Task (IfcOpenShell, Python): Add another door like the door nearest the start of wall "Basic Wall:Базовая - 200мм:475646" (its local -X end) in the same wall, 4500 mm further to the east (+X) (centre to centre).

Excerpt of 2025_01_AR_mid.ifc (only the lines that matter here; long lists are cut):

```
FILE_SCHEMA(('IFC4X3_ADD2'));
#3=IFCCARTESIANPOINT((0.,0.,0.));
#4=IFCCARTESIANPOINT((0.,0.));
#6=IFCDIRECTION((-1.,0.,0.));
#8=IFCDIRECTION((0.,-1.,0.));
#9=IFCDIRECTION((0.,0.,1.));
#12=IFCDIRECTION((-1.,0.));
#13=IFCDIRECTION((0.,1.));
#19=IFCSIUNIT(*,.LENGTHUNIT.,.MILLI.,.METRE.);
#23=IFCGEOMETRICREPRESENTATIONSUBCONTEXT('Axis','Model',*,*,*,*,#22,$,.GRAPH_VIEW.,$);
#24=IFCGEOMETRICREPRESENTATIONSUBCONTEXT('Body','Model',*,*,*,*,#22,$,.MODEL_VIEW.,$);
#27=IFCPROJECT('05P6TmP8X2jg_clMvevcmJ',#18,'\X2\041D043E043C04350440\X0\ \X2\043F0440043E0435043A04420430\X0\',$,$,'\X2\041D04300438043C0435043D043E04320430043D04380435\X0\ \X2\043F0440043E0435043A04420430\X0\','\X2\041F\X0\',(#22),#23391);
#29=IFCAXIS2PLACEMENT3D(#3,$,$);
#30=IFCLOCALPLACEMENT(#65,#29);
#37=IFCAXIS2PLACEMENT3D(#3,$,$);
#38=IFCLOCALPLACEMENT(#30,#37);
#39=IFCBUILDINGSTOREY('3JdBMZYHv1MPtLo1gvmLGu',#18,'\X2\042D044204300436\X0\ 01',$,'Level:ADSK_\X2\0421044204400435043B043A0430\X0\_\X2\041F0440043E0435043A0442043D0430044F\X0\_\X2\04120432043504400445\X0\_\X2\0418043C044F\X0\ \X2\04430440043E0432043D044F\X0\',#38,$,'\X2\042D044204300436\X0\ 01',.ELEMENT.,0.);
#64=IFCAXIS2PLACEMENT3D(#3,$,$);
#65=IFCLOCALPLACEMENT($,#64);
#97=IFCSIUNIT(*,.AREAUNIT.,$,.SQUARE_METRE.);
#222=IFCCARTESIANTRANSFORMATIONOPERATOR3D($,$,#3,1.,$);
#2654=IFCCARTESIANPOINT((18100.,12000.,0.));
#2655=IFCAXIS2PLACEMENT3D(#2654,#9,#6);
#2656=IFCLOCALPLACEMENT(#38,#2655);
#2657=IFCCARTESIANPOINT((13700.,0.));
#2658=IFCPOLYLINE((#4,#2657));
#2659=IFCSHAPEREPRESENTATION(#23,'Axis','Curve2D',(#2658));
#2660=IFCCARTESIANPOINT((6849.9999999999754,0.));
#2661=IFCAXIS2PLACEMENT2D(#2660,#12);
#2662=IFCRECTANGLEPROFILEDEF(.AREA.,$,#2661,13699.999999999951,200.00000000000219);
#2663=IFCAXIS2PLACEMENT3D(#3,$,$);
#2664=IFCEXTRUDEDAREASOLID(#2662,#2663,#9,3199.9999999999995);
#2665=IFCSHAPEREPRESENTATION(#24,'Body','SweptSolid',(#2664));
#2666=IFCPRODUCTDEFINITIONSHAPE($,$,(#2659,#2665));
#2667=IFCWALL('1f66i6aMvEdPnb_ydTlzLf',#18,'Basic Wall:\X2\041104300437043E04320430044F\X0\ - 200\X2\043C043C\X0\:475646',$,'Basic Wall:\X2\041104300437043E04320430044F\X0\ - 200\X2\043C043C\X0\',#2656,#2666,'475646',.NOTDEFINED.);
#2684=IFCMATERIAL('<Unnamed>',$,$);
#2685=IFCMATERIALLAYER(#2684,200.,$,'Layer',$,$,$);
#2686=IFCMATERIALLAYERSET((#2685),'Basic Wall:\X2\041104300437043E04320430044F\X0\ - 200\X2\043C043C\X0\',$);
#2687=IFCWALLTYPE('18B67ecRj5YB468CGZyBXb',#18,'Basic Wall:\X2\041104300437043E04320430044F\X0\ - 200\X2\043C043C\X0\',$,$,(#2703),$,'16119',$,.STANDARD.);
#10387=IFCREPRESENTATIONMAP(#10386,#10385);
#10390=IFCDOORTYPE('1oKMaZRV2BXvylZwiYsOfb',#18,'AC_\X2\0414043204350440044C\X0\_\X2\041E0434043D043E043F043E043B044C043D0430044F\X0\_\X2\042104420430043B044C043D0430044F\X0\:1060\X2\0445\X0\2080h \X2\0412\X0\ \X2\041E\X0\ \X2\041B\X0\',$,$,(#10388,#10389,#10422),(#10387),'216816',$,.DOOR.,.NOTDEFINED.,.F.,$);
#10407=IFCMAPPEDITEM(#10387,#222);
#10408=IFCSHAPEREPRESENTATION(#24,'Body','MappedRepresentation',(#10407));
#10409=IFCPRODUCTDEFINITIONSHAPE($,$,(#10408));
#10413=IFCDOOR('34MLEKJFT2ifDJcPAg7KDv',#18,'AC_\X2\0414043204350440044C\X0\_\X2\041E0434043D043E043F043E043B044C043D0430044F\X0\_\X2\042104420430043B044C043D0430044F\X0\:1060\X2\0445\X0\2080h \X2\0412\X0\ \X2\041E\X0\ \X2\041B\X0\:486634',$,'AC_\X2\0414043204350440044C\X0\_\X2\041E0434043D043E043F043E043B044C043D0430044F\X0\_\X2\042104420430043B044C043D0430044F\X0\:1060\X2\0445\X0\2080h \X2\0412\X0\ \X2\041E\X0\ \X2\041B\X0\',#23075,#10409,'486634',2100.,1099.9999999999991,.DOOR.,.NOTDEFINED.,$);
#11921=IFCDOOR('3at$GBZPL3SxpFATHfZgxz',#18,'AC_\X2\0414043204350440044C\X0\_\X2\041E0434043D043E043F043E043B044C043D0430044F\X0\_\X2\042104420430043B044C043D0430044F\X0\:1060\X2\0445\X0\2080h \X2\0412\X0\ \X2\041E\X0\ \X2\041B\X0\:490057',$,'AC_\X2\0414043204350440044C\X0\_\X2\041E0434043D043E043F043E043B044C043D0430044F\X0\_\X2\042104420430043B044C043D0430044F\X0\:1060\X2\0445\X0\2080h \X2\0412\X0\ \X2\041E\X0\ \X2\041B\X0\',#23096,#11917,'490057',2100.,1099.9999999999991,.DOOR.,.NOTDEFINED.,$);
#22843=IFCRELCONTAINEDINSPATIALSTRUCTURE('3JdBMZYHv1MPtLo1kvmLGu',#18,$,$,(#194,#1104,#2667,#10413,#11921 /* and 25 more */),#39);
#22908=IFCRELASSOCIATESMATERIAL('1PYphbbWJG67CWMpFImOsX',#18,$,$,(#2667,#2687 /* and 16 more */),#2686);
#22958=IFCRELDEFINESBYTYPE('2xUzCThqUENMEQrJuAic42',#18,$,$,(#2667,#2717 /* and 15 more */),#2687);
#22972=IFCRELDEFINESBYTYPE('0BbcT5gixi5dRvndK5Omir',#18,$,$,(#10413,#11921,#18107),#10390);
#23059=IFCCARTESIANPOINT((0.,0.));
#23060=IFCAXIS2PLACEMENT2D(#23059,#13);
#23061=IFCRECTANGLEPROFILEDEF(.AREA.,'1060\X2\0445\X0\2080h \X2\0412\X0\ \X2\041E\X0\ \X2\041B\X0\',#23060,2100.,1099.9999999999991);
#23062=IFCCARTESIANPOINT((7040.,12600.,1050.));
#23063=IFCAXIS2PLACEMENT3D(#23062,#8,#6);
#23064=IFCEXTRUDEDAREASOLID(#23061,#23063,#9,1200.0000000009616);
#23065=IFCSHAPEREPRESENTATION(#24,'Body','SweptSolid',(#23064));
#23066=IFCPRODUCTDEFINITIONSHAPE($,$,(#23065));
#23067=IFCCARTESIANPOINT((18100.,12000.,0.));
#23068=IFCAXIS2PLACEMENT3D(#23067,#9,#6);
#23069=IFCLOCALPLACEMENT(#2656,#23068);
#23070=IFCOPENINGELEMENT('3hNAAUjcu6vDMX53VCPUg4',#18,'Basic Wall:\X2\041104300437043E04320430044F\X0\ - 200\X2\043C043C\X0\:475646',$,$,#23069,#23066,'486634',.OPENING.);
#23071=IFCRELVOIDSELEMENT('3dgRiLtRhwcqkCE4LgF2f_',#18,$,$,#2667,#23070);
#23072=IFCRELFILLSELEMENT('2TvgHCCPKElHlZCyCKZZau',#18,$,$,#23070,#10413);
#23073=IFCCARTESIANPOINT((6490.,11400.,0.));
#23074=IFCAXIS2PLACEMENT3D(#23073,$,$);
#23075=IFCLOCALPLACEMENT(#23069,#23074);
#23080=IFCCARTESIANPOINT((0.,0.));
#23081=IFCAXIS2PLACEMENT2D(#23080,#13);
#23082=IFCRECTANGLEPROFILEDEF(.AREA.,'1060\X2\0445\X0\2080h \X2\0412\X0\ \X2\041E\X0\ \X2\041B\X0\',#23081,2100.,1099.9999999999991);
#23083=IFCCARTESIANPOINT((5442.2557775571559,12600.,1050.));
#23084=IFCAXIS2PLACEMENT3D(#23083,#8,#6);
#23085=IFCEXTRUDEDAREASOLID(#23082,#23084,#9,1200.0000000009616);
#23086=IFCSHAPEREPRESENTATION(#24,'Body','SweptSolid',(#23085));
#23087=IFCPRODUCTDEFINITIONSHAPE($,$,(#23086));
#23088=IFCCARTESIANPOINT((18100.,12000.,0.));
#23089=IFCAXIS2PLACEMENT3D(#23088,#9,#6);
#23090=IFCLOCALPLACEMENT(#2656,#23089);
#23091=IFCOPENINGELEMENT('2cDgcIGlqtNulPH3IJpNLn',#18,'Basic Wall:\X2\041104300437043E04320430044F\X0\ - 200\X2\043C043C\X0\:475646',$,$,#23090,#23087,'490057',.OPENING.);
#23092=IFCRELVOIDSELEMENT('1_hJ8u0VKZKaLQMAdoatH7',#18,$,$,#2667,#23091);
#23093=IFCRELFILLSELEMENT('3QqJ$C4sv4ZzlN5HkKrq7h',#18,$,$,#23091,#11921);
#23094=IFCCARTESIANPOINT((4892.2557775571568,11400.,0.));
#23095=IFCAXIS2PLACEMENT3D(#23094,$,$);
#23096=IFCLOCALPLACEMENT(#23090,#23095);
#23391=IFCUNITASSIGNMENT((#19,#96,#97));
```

```python
import ifcopenshell
import ifcopenshell.api.feature
import ifcopenshell.api.geometry
import ifcopenshell.api.root
import ifcopenshell.geom
import ifcopenshell.util.element
import ifcopenshell.util.placement
import ifcopenshell.util.shape

model = ifcopenshell.open("2025_01_AR_mid.ifc")
settings = ifcopenshell.geom.settings()


def volume(element):
    """Net volume in cubic metres, openings subtracted."""
    shape = ifcopenshell.geom.create_shape(settings, element)
    return ifcopenshell.util.shape.get_volume(shape.geometry)


def reuse_history(source, copy):
    """copy_class also copies each property set's owner history, people and application; keep the originals."""
    for rel in copy.IsDefinedBy:
        if rel.is_a("IfcRelDefinesByProperties") and (history := rel.RelatingPropertyDefinition.OwnerHistory):
            rel.RelatingPropertyDefinition.OwnerHistory = source.OwnerHistory
            ifcopenshell.util.element.remove_deep2(model, history)


door = model.by_guid("34MLEKJFT2ifDJcPAg7KDv")
opening = door.FillsVoids[0].RelatingOpeningElement
wall = opening.VoidsElements[0].RelatingBuildingElement
before = volume(wall)
shift = ifcopenshell.util.placement.get_local_placement(wall.ObjectPlacement)[:3, 0] * -4500.0

# copy_class copies the void relationship, type, container and properties, but no geometry.
new_opening = ifcopenshell.api.root.copy_class(model, product=opening)
new_opening.Representation = ifcopenshell.util.element.copy_deep(
    model, opening.Representation, exclude=["IfcGeometricRepresentationContext", "IfcRepresentationMap"]
)
new_opening.Name = "Basic Wall:Базовая - 200мм"
new_opening.Tag = None
new_door = ifcopenshell.api.root.copy_class(model, product=door)
new_door.Representation = ifcopenshell.util.element.copy_deep(
    model, door.Representation, exclude=["IfcGeometricRepresentationContext", "IfcRepresentationMap"]
)
new_door.Name = "AC_Дверь_Однопольная_Стальная:1060х2080h В О Л"
new_door.Tag = None
reuse_history(door, new_door)
ifcopenshell.api.feature.add_filling(model, opening=new_opening, element=new_door)

for old, new in ((opening, new_opening), (door, new_door)):
    matrix = ifcopenshell.util.placement.get_local_placement(old.ObjectPlacement)
    matrix[:3, 3] += shift
    ifcopenshell.api.geometry.edit_object_placement(model, product=new, matrix=matrix, is_si=False)

after = volume(wall)

print(f"wall volume {before:.3f} -> {after:.3f} m3")

model.write("2025_01_AR_mid_rev.ifc")
```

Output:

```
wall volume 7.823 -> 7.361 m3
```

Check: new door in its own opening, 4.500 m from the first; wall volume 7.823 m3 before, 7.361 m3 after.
